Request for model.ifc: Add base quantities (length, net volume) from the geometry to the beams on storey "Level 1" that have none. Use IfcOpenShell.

First a look at what the model holds.

```python
import ifcopenshell
import ifcopenshell.util.element
import ifcopenshell.util.unit

model = ifcopenshell.open("model.ifc")
print(model.schema)
for unit_type in ("LENGTHUNIT", "AREAUNIT", "VOLUMEUNIT"):
    print(unit_type, ifcopenshell.util.unit.calculate_unit_scale(model, unit_type))
storey = next(s for s in model.by_type("IfcBuildingStorey") if s.Name == "Level 1")
beams = [e for e in ifcopenshell.util.element.get_decomposition(storey) if e.is_a("IfcBeam")]
for e in sorted(beams, key=lambda e: e.id()):
    print(e.id(), e.is_a(), e.Name, list(ifcopenshell.util.element.get_psets(e, qtos_only=True)), sep=" | ")
```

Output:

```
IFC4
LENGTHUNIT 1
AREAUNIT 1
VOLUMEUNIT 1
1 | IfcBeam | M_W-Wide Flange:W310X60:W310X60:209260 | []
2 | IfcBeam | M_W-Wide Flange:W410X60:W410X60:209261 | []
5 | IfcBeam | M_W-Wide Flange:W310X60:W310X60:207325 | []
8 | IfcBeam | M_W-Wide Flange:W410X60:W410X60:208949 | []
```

```python
import ifcopenshell
import ifcopenshell.api.pset
import ifcopenshell.geom
import ifcopenshell.util.element
import ifcopenshell.util.shape
import ifcopenshell.util.unit

model = ifcopenshell.open("model.ifc")
unit_scale = ifcopenshell.util.unit.calculate_unit_scale(model)
volume_scale = ifcopenshell.util.unit.calculate_unit_scale(model, "VOLUMEUNIT")
settings = ifcopenshell.geom.settings()

storey = next(s for s in model.by_type("IfcBuildingStorey") if s.Name == "Level 1")
beams = [e for e in ifcopenshell.util.element.get_decomposition(storey) if e.is_a("IfcBeam")]

for e in sorted(beams, key=lambda e: e.id()):
    if ifcopenshell.util.element.get_psets(e, qtos_only=True, should_inherit=False):
        continue
    # Geometry comes back in metres, in the element's own axes.
    shape = ifcopenshell.geom.create_shape(settings, e)
    values = {
        "Length": ifcopenshell.util.shape.get_max_xyz(shape.geometry) / unit_scale,
        "NetVolume": ifcopenshell.util.shape.get_volume(shape.geometry) / volume_scale,
    }
    qto = ifcopenshell.api.pset.add_qto(model, product=e, name="Qto_BeamBaseQuantities")
    ifcopenshell.api.pset.edit_qto(model, qto=qto, properties=values)
    print(e.id(), {k: round(v, 3) for k, v in values.items()})

model.write("model_rev.ifc")
```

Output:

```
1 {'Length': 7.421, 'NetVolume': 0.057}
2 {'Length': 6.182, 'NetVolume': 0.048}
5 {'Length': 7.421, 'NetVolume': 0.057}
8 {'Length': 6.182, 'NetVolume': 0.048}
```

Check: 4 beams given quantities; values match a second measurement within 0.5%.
